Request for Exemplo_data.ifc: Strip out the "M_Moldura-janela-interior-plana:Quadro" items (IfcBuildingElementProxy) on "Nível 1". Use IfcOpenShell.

First a look at what the model holds.

```python
import ifcopenshell
import ifcopenshell.util.element

model = ifcopenshell.open("Exemplo_data.ifc")
print(model.schema)
storey = next(s for s in model.by_type("IfcBuildingStorey") if s.Name == "Nível 1")
proxies = [e for e in ifcopenshell.util.element.get_decomposition(storey) if e.is_a("IfcBuildingElementProxy")]
seen = {}
for e in proxies:
    element_type = ifcopenshell.util.element.get_type(e)
    name = element_type.Name if element_type not in (None, e) else None
    seen[name] = seen.get(name, 0) + 1
for name, count in sorted(seen.items(), key=str):
    print(count, "x", name)
```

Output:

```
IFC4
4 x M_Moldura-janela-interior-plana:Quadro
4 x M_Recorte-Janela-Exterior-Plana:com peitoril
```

```python
import ifcopenshell
import ifcopenshell.api.root
import ifcopenshell.util.element

model = ifcopenshell.open("Exemplo_data.ifc")

storey = next(s for s in model.by_type("IfcBuildingStorey") if s.Name == "Nível 1")
proxies = [e for e in ifcopenshell.util.element.get_decomposition(storey) if e.is_a("IfcBuildingElementProxy")]
targets = [e for e in proxies if (t := ifcopenshell.util.element.get_type(e)) not in (None, e) and t.Name == "M_Moldura-janela-interior-plana:Quadro"]

for e in targets:
    ifcopenshell.api.root.remove_product(model, product=e)
print(len(targets), "removed")

model.write("Exemplo_data_updated.ifc")
```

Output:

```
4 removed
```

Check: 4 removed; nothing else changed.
